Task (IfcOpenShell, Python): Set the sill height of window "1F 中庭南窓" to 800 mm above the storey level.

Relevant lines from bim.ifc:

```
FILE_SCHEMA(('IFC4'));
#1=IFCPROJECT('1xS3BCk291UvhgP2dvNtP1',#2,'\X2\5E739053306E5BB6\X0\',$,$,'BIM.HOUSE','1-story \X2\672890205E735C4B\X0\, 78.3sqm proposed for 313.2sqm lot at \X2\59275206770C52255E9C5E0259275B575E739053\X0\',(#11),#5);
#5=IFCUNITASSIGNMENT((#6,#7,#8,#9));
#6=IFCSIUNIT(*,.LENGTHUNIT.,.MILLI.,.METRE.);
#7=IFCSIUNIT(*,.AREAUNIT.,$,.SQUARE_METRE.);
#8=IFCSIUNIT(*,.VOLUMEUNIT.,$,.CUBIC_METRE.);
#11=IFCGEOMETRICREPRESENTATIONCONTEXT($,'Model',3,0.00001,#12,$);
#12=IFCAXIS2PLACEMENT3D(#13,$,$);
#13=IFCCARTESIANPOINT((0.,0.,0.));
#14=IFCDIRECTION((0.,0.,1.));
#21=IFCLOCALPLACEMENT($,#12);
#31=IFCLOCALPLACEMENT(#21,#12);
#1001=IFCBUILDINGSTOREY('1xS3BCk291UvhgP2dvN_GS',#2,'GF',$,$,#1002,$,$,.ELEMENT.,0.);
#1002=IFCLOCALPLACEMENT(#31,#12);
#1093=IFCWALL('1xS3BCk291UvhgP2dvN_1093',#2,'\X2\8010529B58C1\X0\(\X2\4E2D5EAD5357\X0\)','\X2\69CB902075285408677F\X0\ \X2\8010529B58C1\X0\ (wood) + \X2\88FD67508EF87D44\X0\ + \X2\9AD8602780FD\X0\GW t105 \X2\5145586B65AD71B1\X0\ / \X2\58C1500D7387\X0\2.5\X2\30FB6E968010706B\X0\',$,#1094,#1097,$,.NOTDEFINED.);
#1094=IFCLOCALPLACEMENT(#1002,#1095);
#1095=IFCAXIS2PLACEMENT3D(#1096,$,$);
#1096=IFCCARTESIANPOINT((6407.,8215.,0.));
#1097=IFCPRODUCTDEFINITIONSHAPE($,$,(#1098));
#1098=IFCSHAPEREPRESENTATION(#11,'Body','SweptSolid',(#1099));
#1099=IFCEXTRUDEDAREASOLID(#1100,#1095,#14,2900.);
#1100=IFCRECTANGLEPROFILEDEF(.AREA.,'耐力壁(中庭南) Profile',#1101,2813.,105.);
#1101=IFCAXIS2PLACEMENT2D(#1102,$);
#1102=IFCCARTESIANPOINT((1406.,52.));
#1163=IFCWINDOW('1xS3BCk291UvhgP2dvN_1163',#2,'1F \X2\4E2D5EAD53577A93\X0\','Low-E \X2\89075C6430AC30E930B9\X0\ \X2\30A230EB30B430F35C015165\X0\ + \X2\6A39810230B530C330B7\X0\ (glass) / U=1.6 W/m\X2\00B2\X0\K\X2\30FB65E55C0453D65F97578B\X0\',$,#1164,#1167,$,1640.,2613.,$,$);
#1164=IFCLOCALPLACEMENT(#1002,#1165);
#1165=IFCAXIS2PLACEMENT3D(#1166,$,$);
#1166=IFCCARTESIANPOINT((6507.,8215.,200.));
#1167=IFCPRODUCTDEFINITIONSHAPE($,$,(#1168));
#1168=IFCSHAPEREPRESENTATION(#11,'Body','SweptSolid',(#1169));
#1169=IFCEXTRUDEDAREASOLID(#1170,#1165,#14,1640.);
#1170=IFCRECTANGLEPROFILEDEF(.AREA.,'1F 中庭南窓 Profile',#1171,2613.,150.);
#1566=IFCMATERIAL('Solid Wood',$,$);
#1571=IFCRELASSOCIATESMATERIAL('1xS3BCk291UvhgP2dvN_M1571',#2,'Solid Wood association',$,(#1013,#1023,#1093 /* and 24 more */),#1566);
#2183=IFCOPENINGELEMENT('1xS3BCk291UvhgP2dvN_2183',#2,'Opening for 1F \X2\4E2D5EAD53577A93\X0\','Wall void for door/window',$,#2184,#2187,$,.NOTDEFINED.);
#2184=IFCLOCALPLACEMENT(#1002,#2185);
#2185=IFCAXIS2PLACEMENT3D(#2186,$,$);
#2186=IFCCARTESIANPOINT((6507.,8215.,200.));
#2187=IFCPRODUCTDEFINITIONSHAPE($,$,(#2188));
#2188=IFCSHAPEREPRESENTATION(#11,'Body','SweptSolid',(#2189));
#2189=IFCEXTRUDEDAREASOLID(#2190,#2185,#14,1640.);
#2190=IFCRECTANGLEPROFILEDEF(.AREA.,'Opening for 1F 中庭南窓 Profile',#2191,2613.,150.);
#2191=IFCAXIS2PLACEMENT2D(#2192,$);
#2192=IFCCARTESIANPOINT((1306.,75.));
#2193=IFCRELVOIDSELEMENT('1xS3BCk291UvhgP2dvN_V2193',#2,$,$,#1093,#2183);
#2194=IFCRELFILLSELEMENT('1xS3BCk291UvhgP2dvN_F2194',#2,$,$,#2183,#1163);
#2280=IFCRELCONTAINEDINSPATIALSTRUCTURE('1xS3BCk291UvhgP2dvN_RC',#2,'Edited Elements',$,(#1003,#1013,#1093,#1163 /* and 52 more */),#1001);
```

```python
import numpy as np
import ifcopenshell
import ifcopenshell.api.geometry
import ifcopenshell.geom
import ifcopenshell.util.element
import ifcopenshell.util.placement
import ifcopenshell.util.shape
import ifcopenshell.util.unit

model = ifcopenshell.open("bim.ifc")
unit_scale = ifcopenshell.util.unit.calculate_unit_scale(model)

window = model.by_id(1163)
opening = window.FillsVoids[0].RelatingOpeningElement
storey = ifcopenshell.util.element.get_container(window, ifc_class="IfcBuildingStorey")
level = ifcopenshell.util.placement.get_local_placement(storey.ObjectPlacement)[2, 3]

# The opening's origin need not be at the sill, so measure its lowest point.
shape = ifcopenshell.geom.create_shape(ifcopenshell.geom.settings(), opening)
bottom = ifcopenshell.util.shape.get_shape_bottom_elevation(shape, shape.geometry) / unit_scale
dz = level + 800.0 - bottom

shift = np.array([0.0, 0.0, dz])
# The window is not placed relative to its opening, so move both.
for product in (opening, window):
    matrix = ifcopenshell.util.placement.get_local_placement(product.ObjectPlacement)
    matrix[:3, 3] += shift
    ifcopenshell.api.geometry.edit_object_placement(model, product=product, matrix=matrix, is_si=False)

print(f"moved by {dz * unit_scale:+.3f} m")

model.write("bim_v2.ifc")
```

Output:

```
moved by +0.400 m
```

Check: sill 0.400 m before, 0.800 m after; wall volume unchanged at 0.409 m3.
